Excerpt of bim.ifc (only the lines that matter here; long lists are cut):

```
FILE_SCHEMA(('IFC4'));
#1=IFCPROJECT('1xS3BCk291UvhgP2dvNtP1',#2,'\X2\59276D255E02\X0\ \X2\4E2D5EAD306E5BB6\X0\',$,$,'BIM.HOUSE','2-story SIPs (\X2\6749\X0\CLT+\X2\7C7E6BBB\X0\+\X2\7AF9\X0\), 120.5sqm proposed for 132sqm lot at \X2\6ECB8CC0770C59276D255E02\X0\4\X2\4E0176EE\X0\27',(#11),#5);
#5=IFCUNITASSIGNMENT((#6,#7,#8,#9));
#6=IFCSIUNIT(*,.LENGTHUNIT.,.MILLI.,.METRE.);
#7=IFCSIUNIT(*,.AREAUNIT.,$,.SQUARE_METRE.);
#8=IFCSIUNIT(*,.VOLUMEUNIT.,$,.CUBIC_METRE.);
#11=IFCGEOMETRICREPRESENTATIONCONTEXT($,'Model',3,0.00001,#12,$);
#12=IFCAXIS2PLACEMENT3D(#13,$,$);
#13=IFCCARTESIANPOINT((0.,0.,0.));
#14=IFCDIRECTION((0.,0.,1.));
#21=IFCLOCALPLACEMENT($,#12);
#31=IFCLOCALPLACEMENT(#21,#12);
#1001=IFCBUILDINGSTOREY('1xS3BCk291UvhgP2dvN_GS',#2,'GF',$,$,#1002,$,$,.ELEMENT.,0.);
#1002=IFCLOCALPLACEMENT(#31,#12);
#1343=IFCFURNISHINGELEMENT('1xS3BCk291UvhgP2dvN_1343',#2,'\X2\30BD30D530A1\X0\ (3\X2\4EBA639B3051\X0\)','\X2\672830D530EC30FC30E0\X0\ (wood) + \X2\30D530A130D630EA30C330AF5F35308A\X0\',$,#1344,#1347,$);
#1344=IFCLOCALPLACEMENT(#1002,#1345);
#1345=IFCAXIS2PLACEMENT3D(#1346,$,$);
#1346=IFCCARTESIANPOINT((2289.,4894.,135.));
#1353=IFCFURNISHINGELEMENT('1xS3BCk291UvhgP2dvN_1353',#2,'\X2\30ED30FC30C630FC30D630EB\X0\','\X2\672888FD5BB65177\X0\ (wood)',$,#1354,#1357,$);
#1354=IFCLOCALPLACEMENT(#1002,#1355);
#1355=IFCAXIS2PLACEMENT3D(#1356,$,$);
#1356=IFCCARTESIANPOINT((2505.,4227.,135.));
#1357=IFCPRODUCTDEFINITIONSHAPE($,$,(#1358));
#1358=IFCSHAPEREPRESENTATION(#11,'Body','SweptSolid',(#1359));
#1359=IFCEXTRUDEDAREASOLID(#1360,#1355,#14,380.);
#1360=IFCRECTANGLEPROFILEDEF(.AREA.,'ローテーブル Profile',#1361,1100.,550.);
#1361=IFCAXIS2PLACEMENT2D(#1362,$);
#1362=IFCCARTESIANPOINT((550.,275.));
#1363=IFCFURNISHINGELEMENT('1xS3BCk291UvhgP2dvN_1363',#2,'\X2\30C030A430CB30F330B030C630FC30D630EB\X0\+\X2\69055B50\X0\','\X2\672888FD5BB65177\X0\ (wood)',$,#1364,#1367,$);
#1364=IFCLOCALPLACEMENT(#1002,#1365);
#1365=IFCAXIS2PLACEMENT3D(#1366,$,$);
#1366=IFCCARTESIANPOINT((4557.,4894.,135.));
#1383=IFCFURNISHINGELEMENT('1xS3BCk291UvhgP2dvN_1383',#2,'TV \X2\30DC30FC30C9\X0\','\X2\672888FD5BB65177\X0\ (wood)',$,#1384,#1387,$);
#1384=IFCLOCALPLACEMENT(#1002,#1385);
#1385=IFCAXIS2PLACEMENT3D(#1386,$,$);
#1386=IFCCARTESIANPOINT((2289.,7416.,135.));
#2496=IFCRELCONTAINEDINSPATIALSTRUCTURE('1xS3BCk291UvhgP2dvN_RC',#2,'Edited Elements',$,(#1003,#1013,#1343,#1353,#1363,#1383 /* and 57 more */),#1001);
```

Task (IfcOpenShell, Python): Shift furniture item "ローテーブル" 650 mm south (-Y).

```python
import ifcopenshell
import ifcopenshell.api.geometry
import ifcopenshell.util.placement
import ifcopenshell.util.unit

model = ifcopenshell.open("bim.ifc")
unit_scale = ifcopenshell.util.unit.calculate_unit_scale(model)

item = model.by_id(1353)
matrix = ifcopenshell.util.placement.get_local_placement(item.ObjectPlacement)
matrix[1, 3] -= 0.65 / unit_scale
ifcopenshell.api.geometry.edit_object_placement(model, product=item, matrix=matrix, is_si=False)

print(ifcopenshell.util.placement.get_local_placement(item.ObjectPlacement).round(3) + 0.0)

model.write("bim_v2.ifc")
```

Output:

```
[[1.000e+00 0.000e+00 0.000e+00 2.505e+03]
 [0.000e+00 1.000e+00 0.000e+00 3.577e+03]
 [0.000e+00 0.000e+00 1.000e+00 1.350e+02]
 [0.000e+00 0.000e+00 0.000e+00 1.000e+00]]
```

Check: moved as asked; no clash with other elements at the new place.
